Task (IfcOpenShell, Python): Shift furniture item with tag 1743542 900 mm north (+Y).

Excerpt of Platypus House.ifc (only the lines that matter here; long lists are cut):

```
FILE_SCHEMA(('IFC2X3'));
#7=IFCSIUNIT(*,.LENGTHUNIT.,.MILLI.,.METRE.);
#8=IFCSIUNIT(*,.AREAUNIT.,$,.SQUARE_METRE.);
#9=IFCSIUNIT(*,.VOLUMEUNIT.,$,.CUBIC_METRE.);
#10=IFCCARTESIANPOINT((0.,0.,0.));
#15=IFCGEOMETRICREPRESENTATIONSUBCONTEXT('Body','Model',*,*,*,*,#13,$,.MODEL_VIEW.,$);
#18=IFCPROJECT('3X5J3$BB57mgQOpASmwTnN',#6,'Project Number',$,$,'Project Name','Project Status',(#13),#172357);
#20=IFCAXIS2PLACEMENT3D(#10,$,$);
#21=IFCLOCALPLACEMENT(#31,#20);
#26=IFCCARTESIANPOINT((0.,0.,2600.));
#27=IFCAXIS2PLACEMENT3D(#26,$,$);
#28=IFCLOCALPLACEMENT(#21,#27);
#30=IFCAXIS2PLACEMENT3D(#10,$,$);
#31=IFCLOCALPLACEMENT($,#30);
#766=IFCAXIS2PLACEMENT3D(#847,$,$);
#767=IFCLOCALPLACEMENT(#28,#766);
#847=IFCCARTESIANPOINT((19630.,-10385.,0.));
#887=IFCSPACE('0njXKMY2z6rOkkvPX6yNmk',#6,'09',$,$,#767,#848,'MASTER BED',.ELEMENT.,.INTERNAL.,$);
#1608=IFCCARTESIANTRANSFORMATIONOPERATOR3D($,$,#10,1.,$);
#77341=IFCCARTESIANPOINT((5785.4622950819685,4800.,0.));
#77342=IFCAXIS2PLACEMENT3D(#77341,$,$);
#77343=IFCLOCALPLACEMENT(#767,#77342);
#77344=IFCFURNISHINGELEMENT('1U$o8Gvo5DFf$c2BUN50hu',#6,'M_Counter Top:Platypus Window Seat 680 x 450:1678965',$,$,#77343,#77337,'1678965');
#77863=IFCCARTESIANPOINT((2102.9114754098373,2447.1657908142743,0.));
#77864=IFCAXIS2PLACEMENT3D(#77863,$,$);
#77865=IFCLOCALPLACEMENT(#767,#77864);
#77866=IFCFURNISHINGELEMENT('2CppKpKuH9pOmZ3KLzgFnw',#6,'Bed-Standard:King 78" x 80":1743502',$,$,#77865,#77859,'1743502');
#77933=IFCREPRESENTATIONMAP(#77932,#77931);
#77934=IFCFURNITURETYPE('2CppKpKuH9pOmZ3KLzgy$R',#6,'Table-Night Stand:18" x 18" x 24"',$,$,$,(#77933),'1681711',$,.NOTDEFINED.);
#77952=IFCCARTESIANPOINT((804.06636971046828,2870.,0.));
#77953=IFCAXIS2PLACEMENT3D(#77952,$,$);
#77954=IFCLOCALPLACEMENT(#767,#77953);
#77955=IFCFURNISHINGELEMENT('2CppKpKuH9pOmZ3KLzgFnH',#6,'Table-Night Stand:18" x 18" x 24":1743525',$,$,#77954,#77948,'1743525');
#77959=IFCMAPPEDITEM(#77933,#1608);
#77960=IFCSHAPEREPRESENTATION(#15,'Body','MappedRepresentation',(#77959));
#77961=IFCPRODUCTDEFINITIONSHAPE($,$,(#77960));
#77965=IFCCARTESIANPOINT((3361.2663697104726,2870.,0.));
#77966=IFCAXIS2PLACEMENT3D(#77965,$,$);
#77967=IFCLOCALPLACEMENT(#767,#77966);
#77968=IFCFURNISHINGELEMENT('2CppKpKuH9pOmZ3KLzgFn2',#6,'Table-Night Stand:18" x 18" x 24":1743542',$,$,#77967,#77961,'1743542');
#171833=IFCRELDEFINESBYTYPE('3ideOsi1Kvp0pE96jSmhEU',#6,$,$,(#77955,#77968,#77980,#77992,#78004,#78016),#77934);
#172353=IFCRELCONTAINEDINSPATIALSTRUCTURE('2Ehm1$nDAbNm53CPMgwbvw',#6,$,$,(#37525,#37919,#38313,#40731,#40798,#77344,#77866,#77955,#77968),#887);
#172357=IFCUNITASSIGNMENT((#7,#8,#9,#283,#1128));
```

```python
import ifcopenshell
import ifcopenshell.api.geometry
import ifcopenshell.util.placement
import ifcopenshell.util.unit

model = ifcopenshell.open("Platypus House.ifc")
unit_scale = ifcopenshell.util.unit.calculate_unit_scale(model)

item = model.by_guid("2CppKpKuH9pOmZ3KLzgFn2")
matrix = ifcopenshell.util.placement.get_local_placement(item.ObjectPlacement)
matrix[1, 3] += 0.9 / unit_scale
ifcopenshell.api.geometry.edit_object_placement(model, product=item, matrix=matrix, is_si=False)

print(ifcopenshell.util.placement.get_local_placement(item.ObjectPlacement).round(3) + 0.0)

model.write("Platypus House_rev.ifc")
```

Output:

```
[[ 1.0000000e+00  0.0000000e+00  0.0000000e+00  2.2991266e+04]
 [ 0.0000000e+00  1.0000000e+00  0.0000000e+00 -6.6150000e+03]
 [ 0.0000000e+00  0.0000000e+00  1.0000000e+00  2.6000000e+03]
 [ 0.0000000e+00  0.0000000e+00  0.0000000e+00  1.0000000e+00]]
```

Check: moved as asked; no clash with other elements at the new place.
